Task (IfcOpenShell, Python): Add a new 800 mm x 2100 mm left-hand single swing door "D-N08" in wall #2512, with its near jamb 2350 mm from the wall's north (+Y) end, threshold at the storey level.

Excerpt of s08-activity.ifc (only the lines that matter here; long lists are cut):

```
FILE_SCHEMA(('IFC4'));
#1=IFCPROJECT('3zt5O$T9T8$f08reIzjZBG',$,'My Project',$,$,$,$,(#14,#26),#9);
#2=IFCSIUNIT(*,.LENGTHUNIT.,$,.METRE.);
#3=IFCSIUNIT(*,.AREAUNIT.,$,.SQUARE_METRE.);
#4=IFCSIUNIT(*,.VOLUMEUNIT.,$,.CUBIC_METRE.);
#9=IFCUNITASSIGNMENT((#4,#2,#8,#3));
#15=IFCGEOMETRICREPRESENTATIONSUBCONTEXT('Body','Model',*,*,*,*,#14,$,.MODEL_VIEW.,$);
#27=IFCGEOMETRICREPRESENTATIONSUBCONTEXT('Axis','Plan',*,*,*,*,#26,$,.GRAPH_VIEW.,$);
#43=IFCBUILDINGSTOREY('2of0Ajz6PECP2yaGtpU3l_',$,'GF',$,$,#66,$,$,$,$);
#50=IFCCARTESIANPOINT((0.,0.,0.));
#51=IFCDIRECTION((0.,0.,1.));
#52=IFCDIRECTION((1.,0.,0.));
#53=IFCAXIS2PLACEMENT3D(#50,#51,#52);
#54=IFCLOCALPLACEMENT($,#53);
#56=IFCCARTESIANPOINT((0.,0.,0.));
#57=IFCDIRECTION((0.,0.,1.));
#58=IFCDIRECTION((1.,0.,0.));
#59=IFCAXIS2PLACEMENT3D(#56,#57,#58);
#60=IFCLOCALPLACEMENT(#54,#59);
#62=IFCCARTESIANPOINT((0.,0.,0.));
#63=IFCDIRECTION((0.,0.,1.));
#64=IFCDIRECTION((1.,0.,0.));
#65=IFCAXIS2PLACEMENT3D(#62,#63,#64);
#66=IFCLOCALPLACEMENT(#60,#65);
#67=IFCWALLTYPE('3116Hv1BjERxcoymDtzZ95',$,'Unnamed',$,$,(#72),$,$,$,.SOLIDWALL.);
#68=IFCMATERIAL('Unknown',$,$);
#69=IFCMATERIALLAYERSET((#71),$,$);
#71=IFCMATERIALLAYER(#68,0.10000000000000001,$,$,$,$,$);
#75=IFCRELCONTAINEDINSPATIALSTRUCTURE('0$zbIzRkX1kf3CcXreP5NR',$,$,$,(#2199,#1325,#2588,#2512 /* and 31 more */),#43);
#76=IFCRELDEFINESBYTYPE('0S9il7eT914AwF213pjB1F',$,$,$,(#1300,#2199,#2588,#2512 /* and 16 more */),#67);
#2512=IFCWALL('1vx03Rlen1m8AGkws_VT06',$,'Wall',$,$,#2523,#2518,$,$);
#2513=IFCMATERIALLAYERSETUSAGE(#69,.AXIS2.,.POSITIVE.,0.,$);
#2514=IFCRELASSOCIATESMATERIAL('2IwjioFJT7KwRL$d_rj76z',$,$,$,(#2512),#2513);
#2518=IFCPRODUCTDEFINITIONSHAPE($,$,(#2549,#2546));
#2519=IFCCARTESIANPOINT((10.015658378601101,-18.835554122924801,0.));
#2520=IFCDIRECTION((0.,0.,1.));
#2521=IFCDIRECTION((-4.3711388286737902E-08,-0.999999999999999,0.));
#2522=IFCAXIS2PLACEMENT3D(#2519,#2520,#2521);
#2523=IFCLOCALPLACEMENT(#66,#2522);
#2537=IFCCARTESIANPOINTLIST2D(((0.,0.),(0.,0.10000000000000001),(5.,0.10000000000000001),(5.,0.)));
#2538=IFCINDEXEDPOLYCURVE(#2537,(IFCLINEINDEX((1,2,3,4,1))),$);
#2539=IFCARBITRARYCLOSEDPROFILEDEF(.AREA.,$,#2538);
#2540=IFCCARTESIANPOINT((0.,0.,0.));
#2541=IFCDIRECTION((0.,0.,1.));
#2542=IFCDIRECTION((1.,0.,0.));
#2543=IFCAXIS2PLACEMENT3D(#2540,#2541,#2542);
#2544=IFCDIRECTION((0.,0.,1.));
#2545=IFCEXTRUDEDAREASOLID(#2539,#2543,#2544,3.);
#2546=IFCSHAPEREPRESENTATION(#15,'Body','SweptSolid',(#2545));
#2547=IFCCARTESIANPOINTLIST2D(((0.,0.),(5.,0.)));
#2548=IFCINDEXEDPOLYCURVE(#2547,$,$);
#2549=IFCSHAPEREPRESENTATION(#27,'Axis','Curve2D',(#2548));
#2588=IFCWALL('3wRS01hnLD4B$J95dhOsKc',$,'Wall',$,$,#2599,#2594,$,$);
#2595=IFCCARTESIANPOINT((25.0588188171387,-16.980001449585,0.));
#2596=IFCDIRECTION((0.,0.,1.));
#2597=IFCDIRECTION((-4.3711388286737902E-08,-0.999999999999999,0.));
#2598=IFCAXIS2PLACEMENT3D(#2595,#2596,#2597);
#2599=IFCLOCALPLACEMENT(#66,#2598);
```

```python
import numpy as np
import ifcopenshell
import ifcopenshell.api.feature
import ifcopenshell.api.geometry
import ifcopenshell.api.root
import ifcopenshell.api.spatial
import ifcopenshell.geom
import ifcopenshell.util.element
import ifcopenshell.util.placement
import ifcopenshell.util.representation
import ifcopenshell.util.shape
import ifcopenshell.util.unit

model = ifcopenshell.open("s08-activity.ifc")
unit_scale = ifcopenshell.util.unit.calculate_unit_scale(model)
settings = ifcopenshell.geom.settings()


def volume(element):
    """Net volume in cubic metres, openings subtracted."""
    shape = ifcopenshell.geom.create_shape(settings, element)
    return ifcopenshell.util.shape.get_volume(shape.geometry)


wall = model.by_guid("1vx03Rlen1m8AGkws_VT06")
storey = ifcopenshell.util.element.get_container(wall, ifc_class="IfcBuildingStorey")
context = ifcopenshell.util.representation.get_context(model, "Model", "Body", "MODEL_VIEW")
before = volume(wall)

width, height, from_end, sill = 0.8, 2.1, 2.35, 0.0  # metres

# The wall runs along its own X axis, and the end named is its -X end.
wall_shape = ifcopenshell.geom.create_shape(settings, wall)
x, y, z = ifcopenshell.util.shape.get_vertices(wall_shape.geometry).T
start = x.min() + from_end
face, thickness = float(y.min()), float(y.max() - y.min())
wall_matrix = ifcopenshell.util.placement.get_local_placement(wall.ObjectPlacement)
level = ifcopenshell.util.placement.get_local_placement(storey.ObjectPlacement)[2, 3]


def in_wall(x, y):
    """Placement at x, y metres in the wall's axes, at sill height."""
    matrix = wall_matrix.copy()
    matrix[:, 3] = wall_matrix @ np.array([x / unit_scale, y / unit_scale, 0.0, 1.0])
    matrix[2, 3] = level + sill / unit_scale
    return matrix


# Opening: a box that overshoots both wall faces by 50 mm.
opening = ifcopenshell.api.root.create_entity(model, ifc_class="IfcOpeningElement", predefined_type="OPENING")
box = ifcopenshell.api.geometry.add_wall_representation(
    model, context=context, length=width, height=height, thickness=thickness + 0.1
)
ifcopenshell.api.geometry.assign_representation(model, product=opening, representation=box)
ifcopenshell.api.geometry.edit_object_placement(model, product=opening, matrix=in_wall(start, face - 0.05), is_si=False)
ifcopenshell.api.feature.add_feature(model, feature=opening, element=wall)

door = ifcopenshell.api.root.create_entity(model, ifc_class="IfcDoor", name="D-N08", predefined_type="DOOR")
door.OverallWidth, door.OverallHeight = width / unit_scale, height / unit_scale
door.OperationType = "SINGLE_SWING_LEFT"
body = ifcopenshell.api.geometry.add_door_representation(
    model,
    context=context,
    overall_width=door.OverallWidth,
    overall_height=door.OverallHeight,
    operation_type="SINGLE_SWING_LEFT",
    lining_properties={"LiningDepth": thickness / unit_scale, "ThresholdDepth": thickness / unit_scale},
)
ifcopenshell.api.geometry.assign_representation(model, product=door, representation=body)
ifcopenshell.api.spatial.assign_container(model, products=[door], relating_structure=storey)
ifcopenshell.api.feature.add_filling(model, opening=opening, element=door)

# The lining spans the wall, so the door starts at the wall face.
ifcopenshell.api.geometry.edit_object_placement(model, product=door, matrix=in_wall(start, face), is_si=False)

after = volume(wall)

print(f"wall volume {before:.3f} -> {after:.3f} m3")

model.write("s08-activity_edited.ifc")
```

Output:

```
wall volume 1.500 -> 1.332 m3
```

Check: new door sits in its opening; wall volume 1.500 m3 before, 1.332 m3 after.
